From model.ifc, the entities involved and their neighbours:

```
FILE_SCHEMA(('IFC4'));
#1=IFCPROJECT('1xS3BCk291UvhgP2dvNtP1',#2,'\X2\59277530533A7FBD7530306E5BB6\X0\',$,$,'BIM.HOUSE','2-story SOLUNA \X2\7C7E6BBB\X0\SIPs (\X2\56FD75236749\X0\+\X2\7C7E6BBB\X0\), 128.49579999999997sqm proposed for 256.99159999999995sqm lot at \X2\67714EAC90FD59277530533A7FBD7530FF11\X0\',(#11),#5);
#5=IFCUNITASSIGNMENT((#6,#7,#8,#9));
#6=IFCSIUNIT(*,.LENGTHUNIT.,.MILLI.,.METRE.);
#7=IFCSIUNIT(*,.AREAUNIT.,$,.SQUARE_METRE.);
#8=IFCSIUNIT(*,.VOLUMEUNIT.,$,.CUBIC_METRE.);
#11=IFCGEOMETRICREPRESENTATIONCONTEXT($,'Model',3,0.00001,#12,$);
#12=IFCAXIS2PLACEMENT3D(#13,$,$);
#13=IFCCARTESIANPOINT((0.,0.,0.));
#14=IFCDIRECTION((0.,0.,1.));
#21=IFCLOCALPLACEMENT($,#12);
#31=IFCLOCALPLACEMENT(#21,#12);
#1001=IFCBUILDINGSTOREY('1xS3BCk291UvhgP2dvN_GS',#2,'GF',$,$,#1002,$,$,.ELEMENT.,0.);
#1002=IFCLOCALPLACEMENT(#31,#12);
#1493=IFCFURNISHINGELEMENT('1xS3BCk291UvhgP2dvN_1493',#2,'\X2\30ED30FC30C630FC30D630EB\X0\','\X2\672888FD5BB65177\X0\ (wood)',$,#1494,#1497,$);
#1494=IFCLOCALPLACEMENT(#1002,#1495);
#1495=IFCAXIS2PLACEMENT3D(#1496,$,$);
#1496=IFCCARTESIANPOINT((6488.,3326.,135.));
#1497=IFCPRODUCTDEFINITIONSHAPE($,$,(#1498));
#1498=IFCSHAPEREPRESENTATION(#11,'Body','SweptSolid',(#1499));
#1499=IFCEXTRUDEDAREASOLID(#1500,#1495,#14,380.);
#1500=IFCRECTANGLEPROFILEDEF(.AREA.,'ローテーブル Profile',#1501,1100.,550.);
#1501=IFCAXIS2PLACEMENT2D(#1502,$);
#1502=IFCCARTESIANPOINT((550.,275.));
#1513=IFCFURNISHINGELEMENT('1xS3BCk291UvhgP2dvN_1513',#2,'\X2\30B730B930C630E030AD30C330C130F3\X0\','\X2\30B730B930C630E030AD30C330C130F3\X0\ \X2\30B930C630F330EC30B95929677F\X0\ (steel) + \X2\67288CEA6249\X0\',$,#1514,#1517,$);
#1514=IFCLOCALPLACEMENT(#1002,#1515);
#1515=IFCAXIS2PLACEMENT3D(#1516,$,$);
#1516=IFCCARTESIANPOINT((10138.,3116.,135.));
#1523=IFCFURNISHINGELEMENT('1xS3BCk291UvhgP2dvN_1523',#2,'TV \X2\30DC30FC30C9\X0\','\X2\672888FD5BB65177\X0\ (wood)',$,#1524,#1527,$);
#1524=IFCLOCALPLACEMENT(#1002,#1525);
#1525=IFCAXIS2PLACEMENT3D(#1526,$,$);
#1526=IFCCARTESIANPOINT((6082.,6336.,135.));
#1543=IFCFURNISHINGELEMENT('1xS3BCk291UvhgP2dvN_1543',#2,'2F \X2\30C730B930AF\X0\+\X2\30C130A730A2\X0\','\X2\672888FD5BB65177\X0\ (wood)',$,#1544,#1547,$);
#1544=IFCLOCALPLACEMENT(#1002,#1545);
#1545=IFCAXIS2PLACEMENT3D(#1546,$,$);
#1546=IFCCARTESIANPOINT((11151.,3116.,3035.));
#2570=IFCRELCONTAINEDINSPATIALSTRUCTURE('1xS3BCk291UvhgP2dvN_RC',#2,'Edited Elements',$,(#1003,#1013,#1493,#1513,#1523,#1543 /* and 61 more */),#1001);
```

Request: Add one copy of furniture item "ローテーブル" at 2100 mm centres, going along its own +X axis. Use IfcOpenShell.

```python
import ifcopenshell
import ifcopenshell.api.geometry
import ifcopenshell.api.root
import ifcopenshell.util.element
import ifcopenshell.util.placement
import ifcopenshell.util.unit

model = ifcopenshell.open("model.ifc")
unit_scale = ifcopenshell.util.unit.calculate_unit_scale(model)


def reuse_history(source, copy):
    """copy_class also copies each property set's owner history, people and application; keep the originals."""
    for rel in copy.IsDefinedBy:
        if rel.is_a("IfcRelDefinesByProperties") and (history := rel.RelatingPropertyDefinition.OwnerHistory):
            rel.RelatingPropertyDefinition.OwnerHistory = source.OwnerHistory
            ifcopenshell.util.element.remove_deep2(model, history)


source = model.by_guid("1xS3BCk291UvhgP2dvN_1493")
base = ifcopenshell.util.placement.get_local_placement(source.ObjectPlacement)
step = base[:3, 0] * 2.1 / unit_scale

for i in range(1, 2):
    copy = ifcopenshell.api.root.copy_class(model, product=source)
    copy.Representation = ifcopenshell.util.element.copy_deep(
        model, source.Representation, exclude=["IfcGeometricRepresentationContext", "IfcRepresentationMap"]
    )
    reuse_history(source, copy)
    matrix = base.copy()
    matrix[:3, 3] += i * step
    print("added at", matrix[:3, 3].round(3) + 0.0)
    ifcopenshell.api.geometry.edit_object_placement(model, product=copy, matrix=matrix, is_si=False)

model.write("model_edited.ifc")
```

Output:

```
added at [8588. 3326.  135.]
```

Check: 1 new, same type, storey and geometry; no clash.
